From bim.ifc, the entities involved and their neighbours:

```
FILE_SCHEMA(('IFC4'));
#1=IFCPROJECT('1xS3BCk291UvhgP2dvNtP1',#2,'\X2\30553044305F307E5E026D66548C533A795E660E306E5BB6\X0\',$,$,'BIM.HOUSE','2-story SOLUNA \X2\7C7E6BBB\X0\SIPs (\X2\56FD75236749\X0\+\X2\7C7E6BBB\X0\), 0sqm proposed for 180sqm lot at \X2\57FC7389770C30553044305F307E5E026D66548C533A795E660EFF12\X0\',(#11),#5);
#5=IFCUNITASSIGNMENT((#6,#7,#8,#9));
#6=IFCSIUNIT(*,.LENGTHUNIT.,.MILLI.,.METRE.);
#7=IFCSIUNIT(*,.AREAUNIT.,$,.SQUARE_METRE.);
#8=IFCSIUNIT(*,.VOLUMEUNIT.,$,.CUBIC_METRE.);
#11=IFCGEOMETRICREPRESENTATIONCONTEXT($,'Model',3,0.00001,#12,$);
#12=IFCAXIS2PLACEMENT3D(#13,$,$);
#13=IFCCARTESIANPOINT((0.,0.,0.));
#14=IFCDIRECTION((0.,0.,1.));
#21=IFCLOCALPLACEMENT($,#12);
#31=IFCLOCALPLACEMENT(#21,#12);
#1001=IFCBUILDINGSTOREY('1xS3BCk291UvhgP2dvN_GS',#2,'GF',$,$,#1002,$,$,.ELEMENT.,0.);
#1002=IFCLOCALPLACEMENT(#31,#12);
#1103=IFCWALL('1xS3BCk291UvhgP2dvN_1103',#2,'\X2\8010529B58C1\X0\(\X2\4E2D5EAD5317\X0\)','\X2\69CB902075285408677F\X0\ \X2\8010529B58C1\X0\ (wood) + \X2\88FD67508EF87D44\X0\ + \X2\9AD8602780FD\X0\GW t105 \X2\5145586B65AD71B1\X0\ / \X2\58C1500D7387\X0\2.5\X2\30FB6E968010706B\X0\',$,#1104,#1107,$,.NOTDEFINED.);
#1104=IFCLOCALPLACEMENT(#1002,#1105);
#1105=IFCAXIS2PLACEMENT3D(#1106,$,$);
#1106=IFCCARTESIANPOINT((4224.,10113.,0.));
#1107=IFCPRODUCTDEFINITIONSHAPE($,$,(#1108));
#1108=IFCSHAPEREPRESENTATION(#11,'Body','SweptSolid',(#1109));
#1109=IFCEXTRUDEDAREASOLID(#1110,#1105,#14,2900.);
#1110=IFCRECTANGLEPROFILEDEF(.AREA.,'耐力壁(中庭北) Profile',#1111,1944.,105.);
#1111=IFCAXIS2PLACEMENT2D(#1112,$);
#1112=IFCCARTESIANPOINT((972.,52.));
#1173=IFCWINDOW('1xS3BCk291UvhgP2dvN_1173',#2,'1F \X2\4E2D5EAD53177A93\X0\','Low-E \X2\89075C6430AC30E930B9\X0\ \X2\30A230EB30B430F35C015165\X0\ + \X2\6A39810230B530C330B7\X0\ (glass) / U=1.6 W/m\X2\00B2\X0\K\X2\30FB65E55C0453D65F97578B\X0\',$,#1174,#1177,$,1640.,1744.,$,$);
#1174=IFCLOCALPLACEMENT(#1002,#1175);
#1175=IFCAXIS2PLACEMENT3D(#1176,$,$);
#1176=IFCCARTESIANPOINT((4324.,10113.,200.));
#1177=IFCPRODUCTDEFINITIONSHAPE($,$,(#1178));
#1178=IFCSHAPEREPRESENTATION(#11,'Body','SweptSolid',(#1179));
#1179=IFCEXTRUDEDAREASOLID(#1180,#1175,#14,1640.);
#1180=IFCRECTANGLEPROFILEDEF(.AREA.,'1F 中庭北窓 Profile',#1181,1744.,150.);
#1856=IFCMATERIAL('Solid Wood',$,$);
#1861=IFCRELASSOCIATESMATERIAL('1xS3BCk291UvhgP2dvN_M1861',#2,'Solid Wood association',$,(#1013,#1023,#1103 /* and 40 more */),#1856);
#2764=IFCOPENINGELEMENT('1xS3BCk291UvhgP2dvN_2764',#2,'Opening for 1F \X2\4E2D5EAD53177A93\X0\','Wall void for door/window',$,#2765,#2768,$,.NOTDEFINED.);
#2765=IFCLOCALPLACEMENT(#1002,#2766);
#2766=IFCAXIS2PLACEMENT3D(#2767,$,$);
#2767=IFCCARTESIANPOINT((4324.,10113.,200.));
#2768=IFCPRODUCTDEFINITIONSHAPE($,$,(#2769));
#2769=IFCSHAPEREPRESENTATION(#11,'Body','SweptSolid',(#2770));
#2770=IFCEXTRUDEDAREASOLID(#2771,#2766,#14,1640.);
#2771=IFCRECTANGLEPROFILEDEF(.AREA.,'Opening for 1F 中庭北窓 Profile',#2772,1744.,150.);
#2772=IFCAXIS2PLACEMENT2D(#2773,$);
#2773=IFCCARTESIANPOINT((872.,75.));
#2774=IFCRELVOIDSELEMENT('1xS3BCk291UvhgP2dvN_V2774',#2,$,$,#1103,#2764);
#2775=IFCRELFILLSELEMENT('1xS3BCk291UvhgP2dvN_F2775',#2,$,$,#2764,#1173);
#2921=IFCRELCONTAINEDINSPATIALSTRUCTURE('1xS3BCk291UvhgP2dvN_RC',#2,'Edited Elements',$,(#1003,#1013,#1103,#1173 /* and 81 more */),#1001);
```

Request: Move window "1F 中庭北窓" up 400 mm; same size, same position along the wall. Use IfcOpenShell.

```python
import numpy as np
import ifcopenshell
import ifcopenshell.api.geometry
import ifcopenshell.util.placement
import ifcopenshell.util.unit

model = ifcopenshell.open("bim.ifc")
unit_scale = ifcopenshell.util.unit.calculate_unit_scale(model)

window = model.by_guid("1xS3BCk291UvhgP2dvN_1173")
opening = window.FillsVoids[0].RelatingOpeningElement
dz = 0.4 / unit_scale

shift = np.array([0.0, 0.0, dz])
# The window is not placed relative to its opening, so move both.
for product in (opening, window):
    matrix = ifcopenshell.util.placement.get_local_placement(product.ObjectPlacement)
    matrix[:3, 3] += shift
    ifcopenshell.api.geometry.edit_object_placement(model, product=product, matrix=matrix, is_si=False)

print(f"moved by {dz * unit_scale:+.3f} m")

model.write("bim_v2.ifc")
```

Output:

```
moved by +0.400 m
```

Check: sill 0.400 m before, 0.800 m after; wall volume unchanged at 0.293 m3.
